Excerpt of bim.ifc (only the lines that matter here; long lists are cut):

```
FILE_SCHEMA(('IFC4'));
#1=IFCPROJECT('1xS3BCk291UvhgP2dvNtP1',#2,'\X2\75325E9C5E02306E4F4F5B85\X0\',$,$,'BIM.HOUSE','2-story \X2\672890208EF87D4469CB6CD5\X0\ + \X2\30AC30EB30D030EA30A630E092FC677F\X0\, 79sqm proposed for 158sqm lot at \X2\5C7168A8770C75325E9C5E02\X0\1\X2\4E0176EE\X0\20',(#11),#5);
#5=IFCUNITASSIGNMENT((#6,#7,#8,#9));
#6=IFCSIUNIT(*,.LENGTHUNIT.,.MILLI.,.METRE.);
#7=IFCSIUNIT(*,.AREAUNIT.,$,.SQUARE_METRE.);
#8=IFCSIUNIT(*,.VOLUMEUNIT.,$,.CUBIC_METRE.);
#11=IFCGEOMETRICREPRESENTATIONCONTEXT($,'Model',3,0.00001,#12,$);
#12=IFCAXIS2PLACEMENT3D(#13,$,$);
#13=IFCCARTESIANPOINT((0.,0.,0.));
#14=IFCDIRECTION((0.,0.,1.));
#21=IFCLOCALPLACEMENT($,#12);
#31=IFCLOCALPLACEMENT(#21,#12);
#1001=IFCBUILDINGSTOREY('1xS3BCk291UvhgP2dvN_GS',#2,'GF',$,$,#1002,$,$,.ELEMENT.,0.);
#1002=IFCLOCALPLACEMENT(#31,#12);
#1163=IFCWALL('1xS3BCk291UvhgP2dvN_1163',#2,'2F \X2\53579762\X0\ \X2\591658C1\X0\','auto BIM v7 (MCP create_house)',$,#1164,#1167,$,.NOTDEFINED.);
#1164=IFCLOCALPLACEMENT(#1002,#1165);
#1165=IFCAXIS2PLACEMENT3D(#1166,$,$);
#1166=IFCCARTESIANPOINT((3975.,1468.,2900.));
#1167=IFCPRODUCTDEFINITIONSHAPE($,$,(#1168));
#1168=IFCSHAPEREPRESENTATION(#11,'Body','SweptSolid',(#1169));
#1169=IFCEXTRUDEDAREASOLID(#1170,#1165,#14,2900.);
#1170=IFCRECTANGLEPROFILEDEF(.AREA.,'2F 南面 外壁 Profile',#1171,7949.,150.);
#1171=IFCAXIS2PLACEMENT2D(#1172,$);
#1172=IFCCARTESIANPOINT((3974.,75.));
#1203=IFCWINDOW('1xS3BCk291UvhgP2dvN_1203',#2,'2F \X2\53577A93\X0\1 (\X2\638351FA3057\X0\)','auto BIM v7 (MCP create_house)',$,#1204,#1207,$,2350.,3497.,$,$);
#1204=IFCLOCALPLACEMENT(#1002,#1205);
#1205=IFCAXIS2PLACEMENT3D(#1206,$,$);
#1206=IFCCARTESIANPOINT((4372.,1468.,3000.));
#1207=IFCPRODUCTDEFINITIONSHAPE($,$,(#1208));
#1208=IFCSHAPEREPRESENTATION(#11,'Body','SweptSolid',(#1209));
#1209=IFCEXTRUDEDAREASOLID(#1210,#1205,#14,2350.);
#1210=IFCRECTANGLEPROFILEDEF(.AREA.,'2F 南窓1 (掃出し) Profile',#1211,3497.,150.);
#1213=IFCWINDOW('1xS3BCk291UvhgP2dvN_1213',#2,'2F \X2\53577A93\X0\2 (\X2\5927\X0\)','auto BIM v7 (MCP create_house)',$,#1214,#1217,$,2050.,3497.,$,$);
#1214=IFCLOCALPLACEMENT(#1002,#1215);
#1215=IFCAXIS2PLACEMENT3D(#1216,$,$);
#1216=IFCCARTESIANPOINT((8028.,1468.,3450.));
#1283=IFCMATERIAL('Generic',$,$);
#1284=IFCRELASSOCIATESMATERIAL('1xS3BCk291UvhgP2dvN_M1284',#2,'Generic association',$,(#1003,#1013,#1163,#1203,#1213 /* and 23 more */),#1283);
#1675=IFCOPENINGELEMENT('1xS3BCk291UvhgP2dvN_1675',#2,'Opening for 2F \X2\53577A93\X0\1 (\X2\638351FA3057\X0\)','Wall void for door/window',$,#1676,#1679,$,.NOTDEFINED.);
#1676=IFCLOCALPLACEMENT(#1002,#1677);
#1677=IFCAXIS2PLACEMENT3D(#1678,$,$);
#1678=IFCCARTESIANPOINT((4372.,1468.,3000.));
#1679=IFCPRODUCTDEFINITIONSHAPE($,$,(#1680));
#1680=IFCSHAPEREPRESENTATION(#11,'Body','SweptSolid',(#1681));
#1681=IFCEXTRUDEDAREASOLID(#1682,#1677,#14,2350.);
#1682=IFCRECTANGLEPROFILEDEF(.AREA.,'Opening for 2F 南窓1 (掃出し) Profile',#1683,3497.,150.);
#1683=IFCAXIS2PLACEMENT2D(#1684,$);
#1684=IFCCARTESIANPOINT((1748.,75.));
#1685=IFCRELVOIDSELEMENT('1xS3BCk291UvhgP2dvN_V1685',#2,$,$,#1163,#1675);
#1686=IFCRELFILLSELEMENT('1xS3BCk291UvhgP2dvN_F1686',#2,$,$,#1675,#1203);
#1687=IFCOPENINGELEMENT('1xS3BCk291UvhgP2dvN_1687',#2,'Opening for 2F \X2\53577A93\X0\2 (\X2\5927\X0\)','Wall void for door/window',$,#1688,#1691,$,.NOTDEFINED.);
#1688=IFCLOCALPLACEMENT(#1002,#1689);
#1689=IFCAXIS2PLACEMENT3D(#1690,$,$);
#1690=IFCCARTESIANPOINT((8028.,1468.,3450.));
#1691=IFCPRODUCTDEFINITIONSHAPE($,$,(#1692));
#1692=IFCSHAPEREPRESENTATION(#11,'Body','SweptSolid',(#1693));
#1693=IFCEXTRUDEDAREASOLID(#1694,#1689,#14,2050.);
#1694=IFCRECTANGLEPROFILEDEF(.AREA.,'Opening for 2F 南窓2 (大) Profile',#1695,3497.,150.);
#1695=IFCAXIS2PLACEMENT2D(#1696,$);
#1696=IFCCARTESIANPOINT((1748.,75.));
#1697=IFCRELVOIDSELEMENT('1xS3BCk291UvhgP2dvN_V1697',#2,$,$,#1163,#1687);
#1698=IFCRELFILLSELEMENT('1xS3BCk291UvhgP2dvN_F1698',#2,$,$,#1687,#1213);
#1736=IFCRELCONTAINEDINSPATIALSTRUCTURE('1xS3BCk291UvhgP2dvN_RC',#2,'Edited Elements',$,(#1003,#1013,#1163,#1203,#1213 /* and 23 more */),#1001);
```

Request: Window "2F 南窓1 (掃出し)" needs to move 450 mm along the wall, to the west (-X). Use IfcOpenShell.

```python
import ifcopenshell
import ifcopenshell.api.geometry
import ifcopenshell.util.placement

model = ifcopenshell.open("bim.ifc")

window = model.by_guid("1xS3BCk291UvhgP2dvN_1203")
opening = window.FillsVoids[0].RelatingOpeningElement
wall = opening.VoidsElements[0].RelatingBuildingElement

wall_matrix = ifcopenshell.util.placement.get_local_placement(wall.ObjectPlacement)
shift = wall_matrix[:3, 0] * -450.0
before = ifcopenshell.util.placement.get_local_placement(window.ObjectPlacement)[:3, 3].copy()

# The window is not placed relative to its opening, so move both.
for product in (opening, window):
    matrix = ifcopenshell.util.placement.get_local_placement(product.ObjectPlacement)
    matrix[:3, 3] += shift
    ifcopenshell.api.geometry.edit_object_placement(model, product=product, matrix=matrix, is_si=False)

after = ifcopenshell.util.placement.get_local_placement(window.ObjectPlacement)[:3, 3]
print("window moved by", (after - before).round(3) + 0.0)

model.write("bim_v2.ifc")
```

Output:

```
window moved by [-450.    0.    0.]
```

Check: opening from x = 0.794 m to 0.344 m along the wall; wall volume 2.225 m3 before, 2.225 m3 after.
